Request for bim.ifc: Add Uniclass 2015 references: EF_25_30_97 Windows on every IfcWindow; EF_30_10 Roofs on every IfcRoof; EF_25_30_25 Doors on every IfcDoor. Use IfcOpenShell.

First a look at what the model holds.

```python
import ifcopenshell

model = ifcopenshell.open("bim.ifc")
print(model.schema)
print("classifications:", [c.Name for c in model.by_type("IfcClassification")])
for ifc_class in ("IfcDoor", "IfcRoof", "IfcStair", "IfcWall", "IfcWindow"):
    print(ifc_class, len(model.by_type(ifc_class)))
```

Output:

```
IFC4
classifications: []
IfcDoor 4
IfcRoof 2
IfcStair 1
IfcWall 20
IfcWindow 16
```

```python
import ifcopenshell
import ifcopenshell.api.classification

model = ifcopenshell.open("bim.ifc")

system = ifcopenshell.api.classification.add_classification(model, classification="Uniclass 2015")

codes = {
    "IfcWindow": ("EF_25_30_97", "Windows"),
    "IfcRoof": ("EF_30_10", "Roofs"),
    "IfcDoor": ("EF_25_30_25", "Doors"),
}
for ifc_class, (code, name) in codes.items():
    products = model.by_type(ifc_class)
    ifcopenshell.api.classification.add_reference(
        model, products=products, classification=system, identification=code, name=name
    )
    print(code, len(products))

model.write("bim_edited.ifc")
```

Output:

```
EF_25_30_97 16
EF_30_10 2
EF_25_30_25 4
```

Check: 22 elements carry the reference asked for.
